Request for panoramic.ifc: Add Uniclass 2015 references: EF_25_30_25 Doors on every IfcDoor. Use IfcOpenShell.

First a look at what the model holds.

```python
import ifcopenshell

model = ifcopenshell.open("panoramic.ifc")
print(model.schema)
print("classifications:", [c.Name for c in model.by_type("IfcClassification")])
for ifc_class in ("IfcDoor", "IfcRoof", "IfcStair", "IfcWall", "IfcWindow"):
    print(ifc_class, len(model.by_type(ifc_class)))
```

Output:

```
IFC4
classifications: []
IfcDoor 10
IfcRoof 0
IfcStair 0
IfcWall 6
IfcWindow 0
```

```python
import ifcopenshell
import ifcopenshell.api.classification

model = ifcopenshell.open("panoramic.ifc")

system = ifcopenshell.api.classification.add_classification(model, classification="Uniclass 2015")

codes = {
    "IfcDoor": ("EF_25_30_25", "Doors"),
}
for ifc_class, (code, name) in codes.items():
    products = model.by_type(ifc_class)
    ifcopenshell.api.classification.add_reference(
        model, products=products, classification=system, identification=code, name=name
    )
    print(code, len(products))

model.write("panoramic_v2.ifc")
```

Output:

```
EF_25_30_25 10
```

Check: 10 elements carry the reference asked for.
